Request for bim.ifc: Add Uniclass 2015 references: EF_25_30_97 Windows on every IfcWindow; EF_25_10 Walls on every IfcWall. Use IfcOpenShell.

First a look at what the model holds.

```python
import ifcopenshell

model = ifcopenshell.open("bim.ifc")
print(model.schema)
print("classifications:", [c.Name for c in model.by_type("IfcClassification")])
for ifc_class in ("IfcDoor", "IfcRoof", "IfcStair", "IfcWall", "IfcWindow"):
    print(ifc_class, len(model.by_type(ifc_class)))
```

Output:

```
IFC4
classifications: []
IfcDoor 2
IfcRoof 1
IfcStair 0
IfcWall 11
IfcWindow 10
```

```python
import ifcopenshell
import ifcopenshell.api.classification

model = ifcopenshell.open("bim.ifc")

system = ifcopenshell.api.classification.add_classification(model, classification="Uniclass 2015")

codes = {
    "IfcWindow": ("EF_25_30_97", "Windows"),
    "IfcWall": ("EF_25_10", "Walls"),
}
for ifc_class, (code, name) in codes.items():
    products = model.by_type(ifc_class)
    ifcopenshell.api.classification.add_reference(
        model, products=products, classification=system, identification=code, name=name
    )
    print(code, len(products))

model.write("bim_v2.ifc")
```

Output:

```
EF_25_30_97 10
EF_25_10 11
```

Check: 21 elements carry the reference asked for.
